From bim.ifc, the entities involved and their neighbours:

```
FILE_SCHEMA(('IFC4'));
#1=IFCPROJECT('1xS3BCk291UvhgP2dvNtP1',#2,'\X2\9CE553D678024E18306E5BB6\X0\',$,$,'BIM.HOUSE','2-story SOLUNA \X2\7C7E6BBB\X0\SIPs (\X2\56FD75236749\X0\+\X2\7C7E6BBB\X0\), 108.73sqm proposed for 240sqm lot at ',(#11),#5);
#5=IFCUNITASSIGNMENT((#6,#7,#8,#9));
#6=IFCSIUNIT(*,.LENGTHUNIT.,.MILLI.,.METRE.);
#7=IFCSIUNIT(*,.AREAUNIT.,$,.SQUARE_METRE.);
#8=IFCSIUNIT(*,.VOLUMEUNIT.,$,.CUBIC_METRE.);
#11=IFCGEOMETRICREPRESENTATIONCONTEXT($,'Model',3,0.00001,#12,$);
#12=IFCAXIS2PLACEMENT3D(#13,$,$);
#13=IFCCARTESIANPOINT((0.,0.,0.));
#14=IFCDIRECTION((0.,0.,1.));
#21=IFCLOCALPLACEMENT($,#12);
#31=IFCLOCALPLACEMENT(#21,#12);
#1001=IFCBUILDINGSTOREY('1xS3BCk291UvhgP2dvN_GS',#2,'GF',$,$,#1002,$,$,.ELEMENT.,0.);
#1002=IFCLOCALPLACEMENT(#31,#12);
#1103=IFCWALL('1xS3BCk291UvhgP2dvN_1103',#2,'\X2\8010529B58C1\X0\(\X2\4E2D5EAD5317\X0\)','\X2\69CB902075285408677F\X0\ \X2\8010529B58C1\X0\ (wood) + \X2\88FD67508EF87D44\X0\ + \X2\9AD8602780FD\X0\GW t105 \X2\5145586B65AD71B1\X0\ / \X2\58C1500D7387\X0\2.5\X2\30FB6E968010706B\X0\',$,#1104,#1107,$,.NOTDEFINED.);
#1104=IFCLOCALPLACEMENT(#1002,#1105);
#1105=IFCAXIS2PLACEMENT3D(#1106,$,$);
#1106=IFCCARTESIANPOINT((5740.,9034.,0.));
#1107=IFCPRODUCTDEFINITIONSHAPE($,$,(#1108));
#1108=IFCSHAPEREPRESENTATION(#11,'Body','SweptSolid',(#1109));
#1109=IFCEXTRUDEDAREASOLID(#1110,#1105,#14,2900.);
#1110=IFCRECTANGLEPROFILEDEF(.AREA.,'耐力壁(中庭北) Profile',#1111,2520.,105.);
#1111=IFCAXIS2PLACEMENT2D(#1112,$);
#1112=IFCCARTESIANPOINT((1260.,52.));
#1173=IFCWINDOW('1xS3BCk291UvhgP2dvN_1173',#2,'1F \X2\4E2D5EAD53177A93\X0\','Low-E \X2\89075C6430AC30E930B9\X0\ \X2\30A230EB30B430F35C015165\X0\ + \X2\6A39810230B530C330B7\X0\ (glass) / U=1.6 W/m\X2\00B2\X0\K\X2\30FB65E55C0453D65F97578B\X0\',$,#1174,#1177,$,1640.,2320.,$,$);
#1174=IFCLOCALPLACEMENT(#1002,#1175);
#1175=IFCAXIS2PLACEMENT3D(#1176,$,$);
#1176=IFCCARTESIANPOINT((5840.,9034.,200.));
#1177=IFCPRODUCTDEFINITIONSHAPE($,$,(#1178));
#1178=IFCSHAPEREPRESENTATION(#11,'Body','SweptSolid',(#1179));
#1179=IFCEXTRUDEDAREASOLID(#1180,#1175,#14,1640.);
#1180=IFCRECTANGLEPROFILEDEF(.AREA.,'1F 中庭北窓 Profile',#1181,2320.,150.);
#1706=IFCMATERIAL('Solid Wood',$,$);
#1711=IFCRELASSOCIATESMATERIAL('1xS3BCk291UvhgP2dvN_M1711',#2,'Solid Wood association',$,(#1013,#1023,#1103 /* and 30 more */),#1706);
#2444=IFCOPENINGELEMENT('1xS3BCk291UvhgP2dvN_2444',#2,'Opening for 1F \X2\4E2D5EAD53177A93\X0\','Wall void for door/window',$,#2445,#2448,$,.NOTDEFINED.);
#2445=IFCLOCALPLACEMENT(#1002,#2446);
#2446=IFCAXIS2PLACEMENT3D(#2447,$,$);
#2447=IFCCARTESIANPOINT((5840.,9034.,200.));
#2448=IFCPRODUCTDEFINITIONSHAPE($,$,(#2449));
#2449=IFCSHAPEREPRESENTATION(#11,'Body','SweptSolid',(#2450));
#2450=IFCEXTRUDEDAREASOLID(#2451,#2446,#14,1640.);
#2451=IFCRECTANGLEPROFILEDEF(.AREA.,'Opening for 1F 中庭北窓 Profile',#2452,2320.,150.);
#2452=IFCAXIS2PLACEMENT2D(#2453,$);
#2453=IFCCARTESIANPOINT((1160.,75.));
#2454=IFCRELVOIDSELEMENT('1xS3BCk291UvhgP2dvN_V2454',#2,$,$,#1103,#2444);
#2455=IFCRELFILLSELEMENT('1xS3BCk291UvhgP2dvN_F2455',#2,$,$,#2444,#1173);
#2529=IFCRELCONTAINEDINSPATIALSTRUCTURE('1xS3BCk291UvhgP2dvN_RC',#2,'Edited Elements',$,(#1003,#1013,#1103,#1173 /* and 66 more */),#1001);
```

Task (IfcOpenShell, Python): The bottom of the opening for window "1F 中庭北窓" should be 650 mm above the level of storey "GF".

```python
import numpy as np
import ifcopenshell
import ifcopenshell.api.geometry
import ifcopenshell.geom
import ifcopenshell.util.element
import ifcopenshell.util.placement
import ifcopenshell.util.shape
import ifcopenshell.util.unit

model = ifcopenshell.open("bim.ifc")
unit_scale = ifcopenshell.util.unit.calculate_unit_scale(model)

window = model.by_guid("1xS3BCk291UvhgP2dvN_1173")
opening = window.FillsVoids[0].RelatingOpeningElement
storey = ifcopenshell.util.element.get_container(window, ifc_class="IfcBuildingStorey")
level = ifcopenshell.util.placement.get_local_placement(storey.ObjectPlacement)[2, 3]

# The opening's origin need not be at the sill, so measure its lowest point.
shape = ifcopenshell.geom.create_shape(ifcopenshell.geom.settings(), opening)
bottom = ifcopenshell.util.shape.get_shape_bottom_elevation(shape, shape.geometry) / unit_scale
dz = level + 650.0 - bottom

shift = np.array([0.0, 0.0, dz])
# The window is not placed relative to its opening, so move both.
for product in (opening, window):
    matrix = ifcopenshell.util.placement.get_local_placement(product.ObjectPlacement)
    matrix[:3, 3] += shift
    ifcopenshell.api.geometry.edit_object_placement(model, product=product, matrix=matrix, is_si=False)

print(f"moved by {dz * unit_scale:+.3f} m")

model.write("bim_updated.ifc")
```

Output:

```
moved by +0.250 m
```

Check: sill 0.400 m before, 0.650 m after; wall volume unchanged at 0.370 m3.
